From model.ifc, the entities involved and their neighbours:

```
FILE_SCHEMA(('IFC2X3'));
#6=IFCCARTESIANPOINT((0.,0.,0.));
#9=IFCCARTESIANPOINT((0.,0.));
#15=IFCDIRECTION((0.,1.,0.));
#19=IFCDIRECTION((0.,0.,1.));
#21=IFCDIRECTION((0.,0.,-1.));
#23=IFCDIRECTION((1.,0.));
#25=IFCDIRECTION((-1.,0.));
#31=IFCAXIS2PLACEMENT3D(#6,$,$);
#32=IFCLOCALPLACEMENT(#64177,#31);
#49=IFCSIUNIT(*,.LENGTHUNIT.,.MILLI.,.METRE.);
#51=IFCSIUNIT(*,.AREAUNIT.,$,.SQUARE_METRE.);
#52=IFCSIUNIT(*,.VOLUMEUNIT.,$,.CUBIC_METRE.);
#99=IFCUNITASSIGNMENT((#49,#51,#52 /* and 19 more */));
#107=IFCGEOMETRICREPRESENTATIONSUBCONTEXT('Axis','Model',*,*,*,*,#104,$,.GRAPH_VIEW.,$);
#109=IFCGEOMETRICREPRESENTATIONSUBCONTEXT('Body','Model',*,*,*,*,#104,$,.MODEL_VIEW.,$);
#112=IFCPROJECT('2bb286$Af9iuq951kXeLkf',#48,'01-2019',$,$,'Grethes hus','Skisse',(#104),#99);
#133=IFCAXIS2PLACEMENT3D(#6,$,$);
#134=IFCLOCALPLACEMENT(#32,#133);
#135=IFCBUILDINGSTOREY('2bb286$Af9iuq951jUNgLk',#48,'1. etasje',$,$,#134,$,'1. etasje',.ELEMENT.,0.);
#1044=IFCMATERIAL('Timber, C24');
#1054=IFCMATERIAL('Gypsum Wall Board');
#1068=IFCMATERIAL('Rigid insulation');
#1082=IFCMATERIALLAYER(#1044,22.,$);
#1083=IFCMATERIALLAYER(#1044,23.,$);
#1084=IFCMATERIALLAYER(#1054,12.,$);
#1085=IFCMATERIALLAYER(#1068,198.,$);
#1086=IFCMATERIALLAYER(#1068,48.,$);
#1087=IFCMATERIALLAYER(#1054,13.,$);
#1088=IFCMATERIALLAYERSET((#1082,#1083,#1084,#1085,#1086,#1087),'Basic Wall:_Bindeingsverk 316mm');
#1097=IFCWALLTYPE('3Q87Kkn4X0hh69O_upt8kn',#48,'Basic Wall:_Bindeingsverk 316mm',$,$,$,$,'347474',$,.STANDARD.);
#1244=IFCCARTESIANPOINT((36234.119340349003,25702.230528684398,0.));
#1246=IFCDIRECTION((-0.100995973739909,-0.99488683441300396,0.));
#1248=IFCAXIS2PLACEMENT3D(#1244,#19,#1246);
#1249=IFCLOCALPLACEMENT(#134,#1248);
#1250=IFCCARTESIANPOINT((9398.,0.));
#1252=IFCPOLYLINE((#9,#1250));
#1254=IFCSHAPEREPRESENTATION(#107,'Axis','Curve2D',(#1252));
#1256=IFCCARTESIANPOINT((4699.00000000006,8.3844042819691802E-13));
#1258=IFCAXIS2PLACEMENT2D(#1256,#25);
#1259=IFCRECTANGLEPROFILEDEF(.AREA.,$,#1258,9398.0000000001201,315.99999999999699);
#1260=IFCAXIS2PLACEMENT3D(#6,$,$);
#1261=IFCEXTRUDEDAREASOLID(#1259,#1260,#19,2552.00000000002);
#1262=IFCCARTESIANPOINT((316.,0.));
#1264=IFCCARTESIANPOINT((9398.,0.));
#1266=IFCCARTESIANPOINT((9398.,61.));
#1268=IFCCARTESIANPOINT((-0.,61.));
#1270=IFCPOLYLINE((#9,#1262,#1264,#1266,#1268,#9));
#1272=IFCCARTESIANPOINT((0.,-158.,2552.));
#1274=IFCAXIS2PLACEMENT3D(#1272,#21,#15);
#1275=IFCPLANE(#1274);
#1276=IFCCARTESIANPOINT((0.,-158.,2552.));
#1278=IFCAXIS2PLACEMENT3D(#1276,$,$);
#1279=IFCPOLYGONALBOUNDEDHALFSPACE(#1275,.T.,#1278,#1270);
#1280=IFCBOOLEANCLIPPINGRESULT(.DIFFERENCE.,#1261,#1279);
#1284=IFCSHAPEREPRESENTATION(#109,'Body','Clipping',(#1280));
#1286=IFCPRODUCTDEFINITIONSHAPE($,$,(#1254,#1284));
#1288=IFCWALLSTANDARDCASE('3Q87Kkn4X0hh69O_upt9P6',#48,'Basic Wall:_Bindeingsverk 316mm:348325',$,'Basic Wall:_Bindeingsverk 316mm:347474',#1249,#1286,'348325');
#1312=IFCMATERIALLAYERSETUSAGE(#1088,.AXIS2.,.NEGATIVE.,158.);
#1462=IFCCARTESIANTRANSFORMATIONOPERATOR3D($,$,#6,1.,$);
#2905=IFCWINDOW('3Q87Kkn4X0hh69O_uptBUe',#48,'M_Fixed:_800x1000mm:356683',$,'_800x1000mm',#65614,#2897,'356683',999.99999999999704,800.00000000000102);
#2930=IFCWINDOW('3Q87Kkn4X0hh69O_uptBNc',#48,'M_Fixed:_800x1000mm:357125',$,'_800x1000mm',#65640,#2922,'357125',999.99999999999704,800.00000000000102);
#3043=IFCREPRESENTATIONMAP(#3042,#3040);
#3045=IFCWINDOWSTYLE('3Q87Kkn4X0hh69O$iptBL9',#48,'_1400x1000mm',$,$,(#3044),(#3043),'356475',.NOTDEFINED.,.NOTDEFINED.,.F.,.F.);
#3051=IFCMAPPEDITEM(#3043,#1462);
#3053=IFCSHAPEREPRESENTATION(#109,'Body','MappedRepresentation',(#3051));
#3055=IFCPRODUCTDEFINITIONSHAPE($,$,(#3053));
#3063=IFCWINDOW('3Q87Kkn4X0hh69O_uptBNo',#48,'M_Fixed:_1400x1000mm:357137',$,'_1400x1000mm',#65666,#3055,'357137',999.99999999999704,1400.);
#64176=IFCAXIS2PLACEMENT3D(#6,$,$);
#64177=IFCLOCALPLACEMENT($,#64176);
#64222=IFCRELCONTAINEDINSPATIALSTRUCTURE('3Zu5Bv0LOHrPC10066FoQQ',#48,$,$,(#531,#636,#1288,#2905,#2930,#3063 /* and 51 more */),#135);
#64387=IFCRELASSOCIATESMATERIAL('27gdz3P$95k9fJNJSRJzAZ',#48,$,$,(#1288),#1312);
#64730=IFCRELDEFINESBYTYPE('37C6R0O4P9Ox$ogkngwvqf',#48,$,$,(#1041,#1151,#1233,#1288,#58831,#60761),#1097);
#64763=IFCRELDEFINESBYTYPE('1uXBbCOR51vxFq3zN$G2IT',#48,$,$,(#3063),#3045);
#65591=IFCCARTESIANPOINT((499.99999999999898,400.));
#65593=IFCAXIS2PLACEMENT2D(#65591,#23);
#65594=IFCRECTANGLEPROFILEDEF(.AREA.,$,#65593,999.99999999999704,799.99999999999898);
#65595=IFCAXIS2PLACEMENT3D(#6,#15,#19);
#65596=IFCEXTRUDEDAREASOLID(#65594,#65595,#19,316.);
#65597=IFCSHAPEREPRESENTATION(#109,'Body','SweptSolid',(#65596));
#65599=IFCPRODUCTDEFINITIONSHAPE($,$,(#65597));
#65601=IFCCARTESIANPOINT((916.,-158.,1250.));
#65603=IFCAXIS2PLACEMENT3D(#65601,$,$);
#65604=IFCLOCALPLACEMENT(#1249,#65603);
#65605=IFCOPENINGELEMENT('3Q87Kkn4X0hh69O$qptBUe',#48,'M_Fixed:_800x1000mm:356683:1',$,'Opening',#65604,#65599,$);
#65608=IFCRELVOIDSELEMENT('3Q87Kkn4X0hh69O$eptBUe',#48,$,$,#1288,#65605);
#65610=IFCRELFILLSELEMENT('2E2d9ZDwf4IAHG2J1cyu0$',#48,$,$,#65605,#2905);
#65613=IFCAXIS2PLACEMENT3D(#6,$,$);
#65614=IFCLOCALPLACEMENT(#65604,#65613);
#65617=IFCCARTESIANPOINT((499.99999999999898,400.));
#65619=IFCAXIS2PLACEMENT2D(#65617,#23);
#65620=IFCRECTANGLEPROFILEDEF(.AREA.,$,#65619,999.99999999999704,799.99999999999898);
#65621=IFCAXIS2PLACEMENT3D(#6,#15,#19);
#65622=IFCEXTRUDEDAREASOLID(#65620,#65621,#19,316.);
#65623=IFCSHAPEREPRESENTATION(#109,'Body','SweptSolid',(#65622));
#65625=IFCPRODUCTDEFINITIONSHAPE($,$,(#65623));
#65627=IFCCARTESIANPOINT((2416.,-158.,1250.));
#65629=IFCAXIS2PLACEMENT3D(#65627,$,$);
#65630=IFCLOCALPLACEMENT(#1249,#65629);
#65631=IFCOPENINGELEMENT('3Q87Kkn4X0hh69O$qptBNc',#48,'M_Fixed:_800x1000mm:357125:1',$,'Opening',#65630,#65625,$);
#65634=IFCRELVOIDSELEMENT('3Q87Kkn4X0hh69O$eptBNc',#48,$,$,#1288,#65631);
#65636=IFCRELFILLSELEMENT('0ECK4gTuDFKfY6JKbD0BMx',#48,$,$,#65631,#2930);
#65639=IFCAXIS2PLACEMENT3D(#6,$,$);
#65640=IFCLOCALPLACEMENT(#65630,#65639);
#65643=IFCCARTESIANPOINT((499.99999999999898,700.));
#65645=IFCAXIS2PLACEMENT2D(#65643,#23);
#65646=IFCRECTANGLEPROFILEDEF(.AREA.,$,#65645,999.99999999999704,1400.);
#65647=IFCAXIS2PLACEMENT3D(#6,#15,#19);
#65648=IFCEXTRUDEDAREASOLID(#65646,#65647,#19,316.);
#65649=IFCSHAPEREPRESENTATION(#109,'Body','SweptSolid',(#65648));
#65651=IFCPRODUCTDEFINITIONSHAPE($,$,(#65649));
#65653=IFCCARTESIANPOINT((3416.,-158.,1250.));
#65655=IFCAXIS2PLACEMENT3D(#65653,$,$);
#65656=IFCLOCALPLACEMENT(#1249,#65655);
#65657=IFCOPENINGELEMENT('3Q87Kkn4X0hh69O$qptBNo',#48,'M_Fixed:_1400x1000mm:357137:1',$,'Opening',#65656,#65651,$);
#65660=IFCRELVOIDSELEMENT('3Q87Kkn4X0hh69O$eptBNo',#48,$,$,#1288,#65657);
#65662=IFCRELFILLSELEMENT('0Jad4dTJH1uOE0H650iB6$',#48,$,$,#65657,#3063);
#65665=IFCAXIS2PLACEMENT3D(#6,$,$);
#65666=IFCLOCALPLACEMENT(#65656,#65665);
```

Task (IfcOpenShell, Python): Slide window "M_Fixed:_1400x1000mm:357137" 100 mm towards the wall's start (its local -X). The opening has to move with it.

```python
import ifcopenshell
import ifcopenshell.api.geometry
import ifcopenshell.util.placement
import ifcopenshell.util.unit

model = ifcopenshell.open("model.ifc")
unit_scale = ifcopenshell.util.unit.calculate_unit_scale(model)

window = model.by_guid("3Q87Kkn4X0hh69O_uptBNo")
opening = window.FillsVoids[0].RelatingOpeningElement
wall = opening.VoidsElements[0].RelatingBuildingElement

wall_matrix = ifcopenshell.util.placement.get_local_placement(wall.ObjectPlacement)
shift = wall_matrix[:3, 0] * -0.1 / unit_scale
before = ifcopenshell.util.placement.get_local_placement(window.ObjectPlacement)[:3, 3].copy()

# The window is placed relative to its opening, so it follows when the opening moves.
matrix = ifcopenshell.util.placement.get_local_placement(opening.ObjectPlacement)
matrix[:3, 3] += shift
ifcopenshell.api.geometry.edit_object_placement(
    model, product=opening, matrix=matrix, is_si=False, should_transform_children=True
)

after = ifcopenshell.util.placement.get_local_placement(window.ObjectPlacement)[:3, 3]
print("window moved by", (after - before).round(3) + 0.0)

model.write("model-out.ifc")
```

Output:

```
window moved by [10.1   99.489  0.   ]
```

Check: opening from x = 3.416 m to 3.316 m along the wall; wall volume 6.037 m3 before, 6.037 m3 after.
